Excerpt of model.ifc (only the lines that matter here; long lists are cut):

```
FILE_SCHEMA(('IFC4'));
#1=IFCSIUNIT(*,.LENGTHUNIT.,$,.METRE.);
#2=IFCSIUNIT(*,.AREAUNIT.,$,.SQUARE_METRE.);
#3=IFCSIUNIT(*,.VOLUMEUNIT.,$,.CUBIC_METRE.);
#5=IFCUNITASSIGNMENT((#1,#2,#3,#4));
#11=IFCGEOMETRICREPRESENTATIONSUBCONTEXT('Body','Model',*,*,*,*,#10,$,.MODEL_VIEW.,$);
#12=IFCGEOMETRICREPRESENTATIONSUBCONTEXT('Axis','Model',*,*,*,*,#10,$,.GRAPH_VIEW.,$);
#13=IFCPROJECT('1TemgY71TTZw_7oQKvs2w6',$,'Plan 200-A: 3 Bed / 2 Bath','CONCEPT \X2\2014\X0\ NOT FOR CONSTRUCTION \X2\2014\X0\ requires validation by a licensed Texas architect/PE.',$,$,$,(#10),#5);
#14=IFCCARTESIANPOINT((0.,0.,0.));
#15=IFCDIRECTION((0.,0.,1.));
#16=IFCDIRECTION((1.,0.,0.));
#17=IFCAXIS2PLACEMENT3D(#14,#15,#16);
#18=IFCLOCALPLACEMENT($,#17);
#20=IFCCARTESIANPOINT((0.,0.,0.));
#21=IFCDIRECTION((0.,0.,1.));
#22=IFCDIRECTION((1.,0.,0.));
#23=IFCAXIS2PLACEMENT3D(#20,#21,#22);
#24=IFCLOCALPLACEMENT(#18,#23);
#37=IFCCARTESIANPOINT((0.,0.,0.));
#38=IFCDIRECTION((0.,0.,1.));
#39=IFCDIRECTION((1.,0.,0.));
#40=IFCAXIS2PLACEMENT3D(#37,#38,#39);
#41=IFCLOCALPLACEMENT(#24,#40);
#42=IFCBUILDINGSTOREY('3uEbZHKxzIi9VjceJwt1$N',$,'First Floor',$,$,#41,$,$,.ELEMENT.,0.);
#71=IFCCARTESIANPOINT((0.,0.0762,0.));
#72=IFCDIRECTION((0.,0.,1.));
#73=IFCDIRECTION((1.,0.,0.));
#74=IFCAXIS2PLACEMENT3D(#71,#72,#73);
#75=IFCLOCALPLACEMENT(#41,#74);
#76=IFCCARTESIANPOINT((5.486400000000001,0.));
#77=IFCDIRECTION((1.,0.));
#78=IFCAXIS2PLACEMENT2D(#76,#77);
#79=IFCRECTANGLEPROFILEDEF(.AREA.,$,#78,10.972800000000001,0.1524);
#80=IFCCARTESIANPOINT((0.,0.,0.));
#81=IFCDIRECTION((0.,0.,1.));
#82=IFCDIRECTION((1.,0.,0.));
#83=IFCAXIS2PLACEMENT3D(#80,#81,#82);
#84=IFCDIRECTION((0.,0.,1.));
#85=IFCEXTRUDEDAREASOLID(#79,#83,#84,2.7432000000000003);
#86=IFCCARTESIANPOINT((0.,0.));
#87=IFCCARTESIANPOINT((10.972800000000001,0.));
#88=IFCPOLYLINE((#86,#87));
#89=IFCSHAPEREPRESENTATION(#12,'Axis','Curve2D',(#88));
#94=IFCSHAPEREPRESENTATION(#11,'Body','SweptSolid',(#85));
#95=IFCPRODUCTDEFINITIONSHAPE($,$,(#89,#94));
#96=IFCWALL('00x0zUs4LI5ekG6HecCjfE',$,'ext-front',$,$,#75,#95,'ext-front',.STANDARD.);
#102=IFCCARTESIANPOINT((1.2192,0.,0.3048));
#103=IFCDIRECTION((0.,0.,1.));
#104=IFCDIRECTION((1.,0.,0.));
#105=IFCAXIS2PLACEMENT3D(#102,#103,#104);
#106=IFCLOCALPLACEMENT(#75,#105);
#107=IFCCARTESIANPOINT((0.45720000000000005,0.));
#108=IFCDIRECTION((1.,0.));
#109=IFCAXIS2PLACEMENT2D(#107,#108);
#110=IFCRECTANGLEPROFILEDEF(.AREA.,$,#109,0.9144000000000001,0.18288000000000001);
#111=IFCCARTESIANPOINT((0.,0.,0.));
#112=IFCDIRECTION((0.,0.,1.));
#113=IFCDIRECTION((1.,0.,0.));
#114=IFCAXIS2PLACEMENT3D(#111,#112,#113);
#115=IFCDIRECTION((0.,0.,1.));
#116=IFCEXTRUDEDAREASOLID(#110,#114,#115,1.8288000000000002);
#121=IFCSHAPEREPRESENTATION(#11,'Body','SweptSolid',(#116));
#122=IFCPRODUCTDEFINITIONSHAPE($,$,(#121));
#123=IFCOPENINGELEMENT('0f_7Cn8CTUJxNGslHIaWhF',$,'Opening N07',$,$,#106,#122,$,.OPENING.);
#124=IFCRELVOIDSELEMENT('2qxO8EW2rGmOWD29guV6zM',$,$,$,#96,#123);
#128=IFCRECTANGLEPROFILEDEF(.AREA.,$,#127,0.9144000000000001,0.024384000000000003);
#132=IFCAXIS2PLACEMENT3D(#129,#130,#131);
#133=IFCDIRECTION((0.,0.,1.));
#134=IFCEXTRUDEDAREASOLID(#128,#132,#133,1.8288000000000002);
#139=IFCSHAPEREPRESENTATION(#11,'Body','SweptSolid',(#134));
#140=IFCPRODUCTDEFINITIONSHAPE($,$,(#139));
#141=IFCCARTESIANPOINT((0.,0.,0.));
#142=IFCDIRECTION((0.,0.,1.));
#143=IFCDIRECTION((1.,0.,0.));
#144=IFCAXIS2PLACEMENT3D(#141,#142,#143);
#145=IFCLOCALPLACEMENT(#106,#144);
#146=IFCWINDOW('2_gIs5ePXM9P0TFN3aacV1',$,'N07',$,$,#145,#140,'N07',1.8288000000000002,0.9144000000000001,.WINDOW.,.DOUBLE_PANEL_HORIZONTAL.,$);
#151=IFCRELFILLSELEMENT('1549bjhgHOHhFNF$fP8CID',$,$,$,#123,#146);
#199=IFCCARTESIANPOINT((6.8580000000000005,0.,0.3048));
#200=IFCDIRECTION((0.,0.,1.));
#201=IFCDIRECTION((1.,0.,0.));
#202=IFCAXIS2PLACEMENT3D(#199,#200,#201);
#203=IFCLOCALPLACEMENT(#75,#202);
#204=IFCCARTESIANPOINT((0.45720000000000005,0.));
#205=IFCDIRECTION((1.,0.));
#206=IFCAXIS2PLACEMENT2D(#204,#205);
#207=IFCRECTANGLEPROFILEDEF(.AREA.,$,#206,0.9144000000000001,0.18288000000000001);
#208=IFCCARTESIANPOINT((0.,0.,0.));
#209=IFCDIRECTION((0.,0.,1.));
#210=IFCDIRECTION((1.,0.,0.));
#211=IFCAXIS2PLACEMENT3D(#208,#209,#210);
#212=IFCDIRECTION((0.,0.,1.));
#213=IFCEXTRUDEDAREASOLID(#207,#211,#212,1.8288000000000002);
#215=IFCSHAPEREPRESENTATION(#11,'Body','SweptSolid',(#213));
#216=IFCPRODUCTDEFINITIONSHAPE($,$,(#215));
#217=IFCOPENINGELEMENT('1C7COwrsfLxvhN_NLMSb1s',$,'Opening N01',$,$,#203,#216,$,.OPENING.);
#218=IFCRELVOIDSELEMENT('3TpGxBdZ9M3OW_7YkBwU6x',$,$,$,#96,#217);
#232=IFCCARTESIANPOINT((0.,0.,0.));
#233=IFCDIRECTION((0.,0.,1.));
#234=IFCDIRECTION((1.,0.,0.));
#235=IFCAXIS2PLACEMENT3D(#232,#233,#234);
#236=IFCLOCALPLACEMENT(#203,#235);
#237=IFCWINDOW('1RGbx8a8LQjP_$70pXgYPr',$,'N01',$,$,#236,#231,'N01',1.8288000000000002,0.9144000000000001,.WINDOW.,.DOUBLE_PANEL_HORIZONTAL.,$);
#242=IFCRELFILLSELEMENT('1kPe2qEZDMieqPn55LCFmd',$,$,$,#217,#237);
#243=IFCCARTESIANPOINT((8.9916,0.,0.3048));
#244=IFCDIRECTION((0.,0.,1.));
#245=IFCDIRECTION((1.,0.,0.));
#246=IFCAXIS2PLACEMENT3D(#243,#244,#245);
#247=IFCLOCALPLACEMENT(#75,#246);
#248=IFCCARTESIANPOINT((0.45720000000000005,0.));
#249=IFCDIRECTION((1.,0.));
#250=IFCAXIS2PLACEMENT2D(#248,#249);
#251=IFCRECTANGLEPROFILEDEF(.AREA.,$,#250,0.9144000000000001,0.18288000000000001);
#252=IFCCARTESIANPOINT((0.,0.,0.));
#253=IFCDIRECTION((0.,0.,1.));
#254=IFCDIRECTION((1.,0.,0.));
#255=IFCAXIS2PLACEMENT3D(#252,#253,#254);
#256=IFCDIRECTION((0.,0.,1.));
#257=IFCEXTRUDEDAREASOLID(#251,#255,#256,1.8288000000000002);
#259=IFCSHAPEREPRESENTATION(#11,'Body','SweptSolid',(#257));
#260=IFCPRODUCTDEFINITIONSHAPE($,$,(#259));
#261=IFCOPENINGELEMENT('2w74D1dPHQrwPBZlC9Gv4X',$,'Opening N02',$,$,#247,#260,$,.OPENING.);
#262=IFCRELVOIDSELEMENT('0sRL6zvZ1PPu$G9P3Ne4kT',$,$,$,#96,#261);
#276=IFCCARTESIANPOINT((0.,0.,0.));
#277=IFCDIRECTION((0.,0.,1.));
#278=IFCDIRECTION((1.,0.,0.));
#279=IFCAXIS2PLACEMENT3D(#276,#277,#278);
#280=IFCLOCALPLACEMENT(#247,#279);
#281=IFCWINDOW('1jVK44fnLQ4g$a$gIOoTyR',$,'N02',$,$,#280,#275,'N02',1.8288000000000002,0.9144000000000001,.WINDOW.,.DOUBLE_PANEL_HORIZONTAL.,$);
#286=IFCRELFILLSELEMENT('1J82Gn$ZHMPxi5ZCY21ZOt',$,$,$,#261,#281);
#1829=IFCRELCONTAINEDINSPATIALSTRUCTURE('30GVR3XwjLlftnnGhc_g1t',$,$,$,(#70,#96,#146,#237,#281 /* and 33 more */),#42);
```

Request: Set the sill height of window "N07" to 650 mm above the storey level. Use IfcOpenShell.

```python
import numpy as np
import ifcopenshell
import ifcopenshell.api.geometry
import ifcopenshell.geom
import ifcopenshell.util.element
import ifcopenshell.util.placement
import ifcopenshell.util.shape
import ifcopenshell.util.unit

model = ifcopenshell.open("model.ifc")
unit_scale = ifcopenshell.util.unit.calculate_unit_scale(model)

window = model.by_guid("2_gIs5ePXM9P0TFN3aacV1")
opening = window.FillsVoids[0].RelatingOpeningElement
storey = ifcopenshell.util.element.get_container(window, ifc_class="IfcBuildingStorey")
level = ifcopenshell.util.placement.get_local_placement(storey.ObjectPlacement)[2, 3]

# The opening's origin need not be at the sill, so measure its lowest point.
shape = ifcopenshell.geom.create_shape(ifcopenshell.geom.settings(), opening)
bottom = ifcopenshell.util.shape.get_shape_bottom_elevation(shape, shape.geometry) / unit_scale
dz = level + 0.65 / unit_scale - bottom

shift = np.array([0.0, 0.0, dz])
# The window is placed relative to its opening, so it follows when the opening moves.
matrix = ifcopenshell.util.placement.get_local_placement(opening.ObjectPlacement)
matrix[:3, 3] += shift
ifcopenshell.api.geometry.edit_object_placement(
    model, product=opening, matrix=matrix, is_si=False, should_transform_children=True
)

print(f"moved by {dz * unit_scale:+.3f} m")

model.write("model_updated.ifc")
```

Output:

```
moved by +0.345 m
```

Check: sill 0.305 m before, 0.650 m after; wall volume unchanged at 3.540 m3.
